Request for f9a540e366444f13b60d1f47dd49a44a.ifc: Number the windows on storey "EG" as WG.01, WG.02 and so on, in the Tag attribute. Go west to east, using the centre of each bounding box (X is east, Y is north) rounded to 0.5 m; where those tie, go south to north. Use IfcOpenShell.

First a look at what the model holds.

```python
import ifcopenshell
import ifcopenshell.util.element
import ifcopenshell.util.placement

model = ifcopenshell.open("f9a540e366444f13b60d1f47dd49a44a.ifc")
print(model.schema)
storey = next(s for s in model.by_type("IfcBuildingStorey") if s.Name == "EG")
windows = [e for e in ifcopenshell.util.element.get_decomposition(storey) if e.is_a("IfcWindow")]
for e in sorted(windows, key=lambda e: e.id()):
    origin = ifcopenshell.util.placement.get_local_placement(e.ObjectPlacement)[:3, 3]
    print(e.id(), e.Tag, e.Name, origin.round(2) + 0.0, sep=" | ")
```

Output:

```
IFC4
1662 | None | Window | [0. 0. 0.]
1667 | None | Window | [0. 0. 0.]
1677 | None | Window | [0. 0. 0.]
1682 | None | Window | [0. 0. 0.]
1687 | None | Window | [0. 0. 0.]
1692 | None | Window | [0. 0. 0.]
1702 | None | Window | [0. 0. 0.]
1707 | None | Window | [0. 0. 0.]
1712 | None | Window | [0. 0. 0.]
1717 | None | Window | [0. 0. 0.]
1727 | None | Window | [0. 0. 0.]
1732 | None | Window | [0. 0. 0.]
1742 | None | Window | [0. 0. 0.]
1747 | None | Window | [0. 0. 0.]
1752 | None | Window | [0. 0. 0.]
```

```python
import ifcopenshell
import ifcopenshell.geom
import ifcopenshell.util.element
import ifcopenshell.util.shape

model = ifcopenshell.open("f9a540e366444f13b60d1f47dd49a44a.ifc")
settings = ifcopenshell.geom.settings()
settings.set("use-world-coords", True)


def centre(element):
    shape = ifcopenshell.geom.create_shape(settings, element)
    return ifcopenshell.util.shape.get_bbox_centroid(shape.geometry)


storey = next(s for s in model.by_type("IfcBuildingStorey") if s.Name == "EG")
windows = [e for e in ifcopenshell.util.element.get_decomposition(storey) if e.is_a("IfcWindow")]

# Insertion points can sit at a corner or the storey origin, so sort by the geometry (in metres).
centres = {e: centre(e) for e in windows}
windows.sort(key=lambda e: (round(centres[e][0] / 0.5), centres[e][1]))

for i, e in enumerate(windows, start=1):
    number = f"WG.{i:02d}"
    e.Tag = number
    print(e.id(), number)

model.write("f9a540e366444f13b60d1f47dd49a44a_edited.ifc")
```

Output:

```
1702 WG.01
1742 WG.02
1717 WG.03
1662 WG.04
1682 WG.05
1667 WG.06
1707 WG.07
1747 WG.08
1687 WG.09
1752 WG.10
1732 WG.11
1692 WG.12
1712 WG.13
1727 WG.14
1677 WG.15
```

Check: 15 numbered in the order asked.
